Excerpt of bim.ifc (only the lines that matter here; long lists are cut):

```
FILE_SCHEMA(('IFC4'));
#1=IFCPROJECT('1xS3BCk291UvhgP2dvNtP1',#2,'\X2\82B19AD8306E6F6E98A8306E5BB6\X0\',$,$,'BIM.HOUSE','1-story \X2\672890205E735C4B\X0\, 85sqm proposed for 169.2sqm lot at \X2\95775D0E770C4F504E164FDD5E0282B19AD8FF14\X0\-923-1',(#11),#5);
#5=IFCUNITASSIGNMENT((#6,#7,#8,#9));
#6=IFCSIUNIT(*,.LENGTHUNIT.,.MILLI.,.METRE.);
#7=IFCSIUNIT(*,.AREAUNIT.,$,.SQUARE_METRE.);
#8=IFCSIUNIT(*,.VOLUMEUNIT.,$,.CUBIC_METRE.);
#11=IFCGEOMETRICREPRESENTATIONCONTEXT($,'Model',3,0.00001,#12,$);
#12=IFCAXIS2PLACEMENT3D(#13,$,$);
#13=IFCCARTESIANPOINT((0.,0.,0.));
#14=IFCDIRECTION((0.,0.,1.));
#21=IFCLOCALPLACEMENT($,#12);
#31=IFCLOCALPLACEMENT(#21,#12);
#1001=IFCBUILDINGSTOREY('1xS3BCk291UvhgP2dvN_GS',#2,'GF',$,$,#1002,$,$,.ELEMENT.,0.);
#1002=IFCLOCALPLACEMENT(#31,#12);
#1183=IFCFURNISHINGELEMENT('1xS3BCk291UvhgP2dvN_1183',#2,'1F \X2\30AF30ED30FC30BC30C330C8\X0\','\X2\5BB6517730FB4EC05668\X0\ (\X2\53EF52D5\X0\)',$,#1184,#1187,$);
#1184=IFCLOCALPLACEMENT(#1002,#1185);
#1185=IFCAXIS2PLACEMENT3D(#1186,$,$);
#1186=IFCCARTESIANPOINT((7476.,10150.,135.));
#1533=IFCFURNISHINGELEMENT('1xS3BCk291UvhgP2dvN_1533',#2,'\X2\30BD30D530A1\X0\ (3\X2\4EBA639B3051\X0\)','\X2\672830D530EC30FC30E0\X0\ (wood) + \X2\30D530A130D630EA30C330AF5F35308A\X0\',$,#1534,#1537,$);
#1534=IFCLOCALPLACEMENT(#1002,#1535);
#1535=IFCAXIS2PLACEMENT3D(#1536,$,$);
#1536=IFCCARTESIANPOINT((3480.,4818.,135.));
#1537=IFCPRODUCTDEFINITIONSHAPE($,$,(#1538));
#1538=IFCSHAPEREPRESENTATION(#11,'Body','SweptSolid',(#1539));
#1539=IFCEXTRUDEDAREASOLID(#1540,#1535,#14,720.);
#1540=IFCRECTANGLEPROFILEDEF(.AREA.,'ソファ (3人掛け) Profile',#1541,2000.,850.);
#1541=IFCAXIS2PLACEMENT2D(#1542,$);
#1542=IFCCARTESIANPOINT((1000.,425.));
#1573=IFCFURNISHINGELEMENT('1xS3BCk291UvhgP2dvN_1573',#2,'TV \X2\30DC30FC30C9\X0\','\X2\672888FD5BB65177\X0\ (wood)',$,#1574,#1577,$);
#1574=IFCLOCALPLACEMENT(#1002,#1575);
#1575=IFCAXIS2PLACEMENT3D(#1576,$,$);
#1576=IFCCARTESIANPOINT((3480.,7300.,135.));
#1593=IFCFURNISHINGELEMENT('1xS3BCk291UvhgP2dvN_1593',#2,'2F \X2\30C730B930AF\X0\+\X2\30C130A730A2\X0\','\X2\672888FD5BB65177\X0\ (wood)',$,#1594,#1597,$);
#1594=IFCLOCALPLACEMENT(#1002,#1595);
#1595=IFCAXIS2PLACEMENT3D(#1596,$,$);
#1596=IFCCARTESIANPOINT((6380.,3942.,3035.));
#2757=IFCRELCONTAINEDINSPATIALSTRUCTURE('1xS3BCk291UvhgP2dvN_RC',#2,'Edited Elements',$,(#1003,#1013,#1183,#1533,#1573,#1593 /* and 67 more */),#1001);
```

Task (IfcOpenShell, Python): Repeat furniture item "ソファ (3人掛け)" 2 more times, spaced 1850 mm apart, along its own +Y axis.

```python
import ifcopenshell
import ifcopenshell.api.geometry
import ifcopenshell.api.root
import ifcopenshell.util.element
import ifcopenshell.util.placement
import ifcopenshell.util.unit

model = ifcopenshell.open("bim.ifc")
unit_scale = ifcopenshell.util.unit.calculate_unit_scale(model)


def reuse_history(source, copy):
    """copy_class also copies each property set's owner history, people and application; keep the originals."""
    for rel in copy.IsDefinedBy:
        if rel.is_a("IfcRelDefinesByProperties") and (history := rel.RelatingPropertyDefinition.OwnerHistory):
            rel.RelatingPropertyDefinition.OwnerHistory = source.OwnerHistory
            ifcopenshell.util.element.remove_deep2(model, history)


source = model.by_guid("1xS3BCk291UvhgP2dvN_1533")
base = ifcopenshell.util.placement.get_local_placement(source.ObjectPlacement)
step = base[:3, 1] * 1.85 / unit_scale

for i in range(1, 3):
    copy = ifcopenshell.api.root.copy_class(model, product=source)
    copy.Representation = ifcopenshell.util.element.copy_deep(
        model, source.Representation, exclude=["IfcGeometricRepresentationContext", "IfcRepresentationMap"]
    )
    reuse_history(source, copy)
    matrix = base.copy()
    matrix[:3, 3] += i * step
    print("added at", matrix[:3, 3].round(3) + 0.0)
    ifcopenshell.api.geometry.edit_object_placement(model, product=copy, matrix=matrix, is_si=False)

model.write("bim-out.ifc")
```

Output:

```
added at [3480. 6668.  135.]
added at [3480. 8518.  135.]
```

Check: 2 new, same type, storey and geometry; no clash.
